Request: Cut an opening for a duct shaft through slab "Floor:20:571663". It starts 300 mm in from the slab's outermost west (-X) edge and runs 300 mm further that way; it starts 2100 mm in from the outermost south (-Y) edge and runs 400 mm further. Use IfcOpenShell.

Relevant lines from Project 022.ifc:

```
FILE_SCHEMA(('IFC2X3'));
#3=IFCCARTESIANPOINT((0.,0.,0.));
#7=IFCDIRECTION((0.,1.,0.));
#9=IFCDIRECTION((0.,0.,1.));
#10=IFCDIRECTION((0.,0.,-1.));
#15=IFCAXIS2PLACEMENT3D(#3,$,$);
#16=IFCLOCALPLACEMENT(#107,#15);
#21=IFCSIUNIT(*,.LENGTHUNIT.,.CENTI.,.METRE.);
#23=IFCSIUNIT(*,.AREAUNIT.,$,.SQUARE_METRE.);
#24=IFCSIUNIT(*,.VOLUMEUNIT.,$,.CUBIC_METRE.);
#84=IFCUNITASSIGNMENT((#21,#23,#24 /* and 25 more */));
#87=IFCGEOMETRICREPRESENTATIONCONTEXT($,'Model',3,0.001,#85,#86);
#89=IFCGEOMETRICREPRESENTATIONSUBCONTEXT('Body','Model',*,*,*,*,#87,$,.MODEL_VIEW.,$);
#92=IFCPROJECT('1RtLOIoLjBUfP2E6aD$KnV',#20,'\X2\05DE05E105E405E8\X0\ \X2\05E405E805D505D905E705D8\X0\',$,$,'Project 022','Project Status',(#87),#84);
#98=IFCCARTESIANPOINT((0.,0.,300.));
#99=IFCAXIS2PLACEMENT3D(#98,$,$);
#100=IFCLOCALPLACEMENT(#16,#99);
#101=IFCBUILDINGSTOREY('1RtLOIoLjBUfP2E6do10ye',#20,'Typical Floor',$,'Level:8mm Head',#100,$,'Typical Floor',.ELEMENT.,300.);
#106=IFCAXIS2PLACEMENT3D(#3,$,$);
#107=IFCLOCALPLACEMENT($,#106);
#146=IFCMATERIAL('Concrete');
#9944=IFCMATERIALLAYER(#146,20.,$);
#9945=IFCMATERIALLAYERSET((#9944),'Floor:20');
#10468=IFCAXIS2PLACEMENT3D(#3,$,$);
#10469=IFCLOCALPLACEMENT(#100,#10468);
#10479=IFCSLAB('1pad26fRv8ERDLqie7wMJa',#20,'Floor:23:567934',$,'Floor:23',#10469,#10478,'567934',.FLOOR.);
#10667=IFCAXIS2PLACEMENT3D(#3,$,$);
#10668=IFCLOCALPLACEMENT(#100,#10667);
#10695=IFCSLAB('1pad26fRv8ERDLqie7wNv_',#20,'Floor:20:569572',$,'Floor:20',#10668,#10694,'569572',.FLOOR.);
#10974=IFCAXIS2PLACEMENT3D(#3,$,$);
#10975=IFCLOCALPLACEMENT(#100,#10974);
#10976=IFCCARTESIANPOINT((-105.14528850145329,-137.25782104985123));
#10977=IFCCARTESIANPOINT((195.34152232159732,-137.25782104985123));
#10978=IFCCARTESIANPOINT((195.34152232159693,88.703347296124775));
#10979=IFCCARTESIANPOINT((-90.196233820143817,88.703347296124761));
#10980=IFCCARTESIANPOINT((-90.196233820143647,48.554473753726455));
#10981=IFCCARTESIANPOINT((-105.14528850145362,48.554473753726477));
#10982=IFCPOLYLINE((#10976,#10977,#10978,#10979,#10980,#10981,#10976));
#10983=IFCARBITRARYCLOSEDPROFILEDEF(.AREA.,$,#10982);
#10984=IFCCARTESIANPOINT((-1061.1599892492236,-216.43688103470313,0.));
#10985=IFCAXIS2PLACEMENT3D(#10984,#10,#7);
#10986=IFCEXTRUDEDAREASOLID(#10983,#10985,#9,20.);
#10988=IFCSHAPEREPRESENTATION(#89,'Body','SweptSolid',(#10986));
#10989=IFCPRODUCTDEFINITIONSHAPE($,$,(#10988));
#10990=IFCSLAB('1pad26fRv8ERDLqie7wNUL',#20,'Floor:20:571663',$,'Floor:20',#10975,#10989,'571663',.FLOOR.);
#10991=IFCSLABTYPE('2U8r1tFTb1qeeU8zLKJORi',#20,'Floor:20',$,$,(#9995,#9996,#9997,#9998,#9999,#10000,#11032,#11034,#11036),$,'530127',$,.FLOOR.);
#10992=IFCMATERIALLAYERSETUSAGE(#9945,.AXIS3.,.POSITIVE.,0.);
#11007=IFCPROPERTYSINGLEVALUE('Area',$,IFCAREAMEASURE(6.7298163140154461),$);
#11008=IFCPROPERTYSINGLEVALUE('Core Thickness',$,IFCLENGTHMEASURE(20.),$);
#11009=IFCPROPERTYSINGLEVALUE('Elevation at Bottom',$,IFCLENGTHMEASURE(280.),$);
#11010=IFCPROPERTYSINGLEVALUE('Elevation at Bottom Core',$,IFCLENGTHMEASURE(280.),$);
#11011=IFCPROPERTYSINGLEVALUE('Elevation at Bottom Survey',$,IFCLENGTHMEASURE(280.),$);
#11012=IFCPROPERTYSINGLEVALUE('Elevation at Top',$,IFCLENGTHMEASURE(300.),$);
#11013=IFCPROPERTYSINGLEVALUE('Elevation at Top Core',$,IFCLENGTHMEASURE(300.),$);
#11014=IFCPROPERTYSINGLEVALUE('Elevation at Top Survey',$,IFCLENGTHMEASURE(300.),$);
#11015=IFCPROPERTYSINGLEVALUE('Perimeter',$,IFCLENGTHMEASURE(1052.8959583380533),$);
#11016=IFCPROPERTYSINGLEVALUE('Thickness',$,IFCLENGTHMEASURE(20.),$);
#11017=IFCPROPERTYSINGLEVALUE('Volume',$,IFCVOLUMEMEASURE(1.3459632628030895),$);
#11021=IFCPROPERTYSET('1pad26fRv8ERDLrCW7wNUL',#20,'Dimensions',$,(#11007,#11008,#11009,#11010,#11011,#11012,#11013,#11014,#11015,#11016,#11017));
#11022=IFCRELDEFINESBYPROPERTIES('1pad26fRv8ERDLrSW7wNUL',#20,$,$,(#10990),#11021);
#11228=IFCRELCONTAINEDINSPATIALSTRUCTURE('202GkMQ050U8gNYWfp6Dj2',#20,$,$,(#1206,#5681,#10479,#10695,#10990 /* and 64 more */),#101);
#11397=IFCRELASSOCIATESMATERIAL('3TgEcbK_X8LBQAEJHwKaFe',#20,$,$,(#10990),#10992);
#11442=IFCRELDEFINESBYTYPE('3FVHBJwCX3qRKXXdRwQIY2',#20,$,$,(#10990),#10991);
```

```python
import numpy as np
import ifcopenshell
import ifcopenshell.api.feature
import ifcopenshell.api.geometry
import ifcopenshell.api.pset
import ifcopenshell.api.root
import ifcopenshell.geom
import ifcopenshell.util.element
import ifcopenshell.util.placement
import ifcopenshell.util.representation
import ifcopenshell.util.shape
import ifcopenshell.util.unit

model = ifcopenshell.open("Project 022.ifc")
unit_scale = ifcopenshell.util.unit.calculate_unit_scale(model)
area_scale = ifcopenshell.util.unit.calculate_unit_scale(model, "AREAUNIT")
volume_scale = ifcopenshell.util.unit.calculate_unit_scale(model, "VOLUMEUNIT")
settings = ifcopenshell.geom.settings()


def volume(element):
    """Net volume in cubic metres, openings subtracted."""
    shape = ifcopenshell.geom.create_shape(settings, element)
    return ifcopenshell.util.shape.get_volume(shape.geometry)


slab = model.by_guid("1pad26fRv8ERDLqie7wNUL")
before = volume(slab)

# Extent in the slab's own axes, in metres. The edges named are its -X and -Y sides.
slab_shape = ifcopenshell.geom.create_shape(settings, slab)
vertices = ifcopenshell.util.shape.get_vertices(slab_shape.geometry)
x_min, y_min, bottom = vertices.min(axis=0)
top = vertices[:, 2].max()

opening = ifcopenshell.api.root.create_entity(model, ifc_class="IfcOpeningElement", name="Duct shaft opening")
context = ifcopenshell.util.representation.get_context(model, "Model", "Body", "MODEL_VIEW")
width, depth = 0.3, 0.4
outline = [(0.0, 0.0), (width, 0.0), (width, depth), (0.0, depth), (0.0, 0.0)]
# Overshoot both faces by 50 mm so the cut is clean.
shape = ifcopenshell.api.geometry.add_slab_representation(
    model, context=context, depth=top - bottom + 0.1, polyline=outline
)
ifcopenshell.api.geometry.assign_representation(model, product=opening, representation=shape)

matrix = ifcopenshell.util.placement.get_local_placement(slab.ObjectPlacement)
matrix[:, 3] = matrix @ np.append(np.array([x_min + 0.3, y_min + 2.1, bottom - 0.05]) / unit_scale, 1.0)
ifcopenshell.api.geometry.edit_object_placement(model, product=opening, matrix=matrix, is_si=False)
ifcopenshell.api.feature.add_feature(model, feature=opening, element=slab)

after = volume(slab)

# Update the slab's stored quantities.
pset = model.by_id(ifcopenshell.util.element.get_pset(slab, "Dimensions", should_inherit=False)["id"])
ifcopenshell.api.pset.edit_pset(model, pset=pset, properties={
    "Area": model.create_entity("IfcAreaMeasure", after / (top - bottom) / area_scale),
    "Volume": model.create_entity("IfcVolumeMeasure", after / volume_scale),
})

print(f"slab volume {before:.3f} -> {after:.3f} m3")

model.write("Project 022_rev.ifc")
```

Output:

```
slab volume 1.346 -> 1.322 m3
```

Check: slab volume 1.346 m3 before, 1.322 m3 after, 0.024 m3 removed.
